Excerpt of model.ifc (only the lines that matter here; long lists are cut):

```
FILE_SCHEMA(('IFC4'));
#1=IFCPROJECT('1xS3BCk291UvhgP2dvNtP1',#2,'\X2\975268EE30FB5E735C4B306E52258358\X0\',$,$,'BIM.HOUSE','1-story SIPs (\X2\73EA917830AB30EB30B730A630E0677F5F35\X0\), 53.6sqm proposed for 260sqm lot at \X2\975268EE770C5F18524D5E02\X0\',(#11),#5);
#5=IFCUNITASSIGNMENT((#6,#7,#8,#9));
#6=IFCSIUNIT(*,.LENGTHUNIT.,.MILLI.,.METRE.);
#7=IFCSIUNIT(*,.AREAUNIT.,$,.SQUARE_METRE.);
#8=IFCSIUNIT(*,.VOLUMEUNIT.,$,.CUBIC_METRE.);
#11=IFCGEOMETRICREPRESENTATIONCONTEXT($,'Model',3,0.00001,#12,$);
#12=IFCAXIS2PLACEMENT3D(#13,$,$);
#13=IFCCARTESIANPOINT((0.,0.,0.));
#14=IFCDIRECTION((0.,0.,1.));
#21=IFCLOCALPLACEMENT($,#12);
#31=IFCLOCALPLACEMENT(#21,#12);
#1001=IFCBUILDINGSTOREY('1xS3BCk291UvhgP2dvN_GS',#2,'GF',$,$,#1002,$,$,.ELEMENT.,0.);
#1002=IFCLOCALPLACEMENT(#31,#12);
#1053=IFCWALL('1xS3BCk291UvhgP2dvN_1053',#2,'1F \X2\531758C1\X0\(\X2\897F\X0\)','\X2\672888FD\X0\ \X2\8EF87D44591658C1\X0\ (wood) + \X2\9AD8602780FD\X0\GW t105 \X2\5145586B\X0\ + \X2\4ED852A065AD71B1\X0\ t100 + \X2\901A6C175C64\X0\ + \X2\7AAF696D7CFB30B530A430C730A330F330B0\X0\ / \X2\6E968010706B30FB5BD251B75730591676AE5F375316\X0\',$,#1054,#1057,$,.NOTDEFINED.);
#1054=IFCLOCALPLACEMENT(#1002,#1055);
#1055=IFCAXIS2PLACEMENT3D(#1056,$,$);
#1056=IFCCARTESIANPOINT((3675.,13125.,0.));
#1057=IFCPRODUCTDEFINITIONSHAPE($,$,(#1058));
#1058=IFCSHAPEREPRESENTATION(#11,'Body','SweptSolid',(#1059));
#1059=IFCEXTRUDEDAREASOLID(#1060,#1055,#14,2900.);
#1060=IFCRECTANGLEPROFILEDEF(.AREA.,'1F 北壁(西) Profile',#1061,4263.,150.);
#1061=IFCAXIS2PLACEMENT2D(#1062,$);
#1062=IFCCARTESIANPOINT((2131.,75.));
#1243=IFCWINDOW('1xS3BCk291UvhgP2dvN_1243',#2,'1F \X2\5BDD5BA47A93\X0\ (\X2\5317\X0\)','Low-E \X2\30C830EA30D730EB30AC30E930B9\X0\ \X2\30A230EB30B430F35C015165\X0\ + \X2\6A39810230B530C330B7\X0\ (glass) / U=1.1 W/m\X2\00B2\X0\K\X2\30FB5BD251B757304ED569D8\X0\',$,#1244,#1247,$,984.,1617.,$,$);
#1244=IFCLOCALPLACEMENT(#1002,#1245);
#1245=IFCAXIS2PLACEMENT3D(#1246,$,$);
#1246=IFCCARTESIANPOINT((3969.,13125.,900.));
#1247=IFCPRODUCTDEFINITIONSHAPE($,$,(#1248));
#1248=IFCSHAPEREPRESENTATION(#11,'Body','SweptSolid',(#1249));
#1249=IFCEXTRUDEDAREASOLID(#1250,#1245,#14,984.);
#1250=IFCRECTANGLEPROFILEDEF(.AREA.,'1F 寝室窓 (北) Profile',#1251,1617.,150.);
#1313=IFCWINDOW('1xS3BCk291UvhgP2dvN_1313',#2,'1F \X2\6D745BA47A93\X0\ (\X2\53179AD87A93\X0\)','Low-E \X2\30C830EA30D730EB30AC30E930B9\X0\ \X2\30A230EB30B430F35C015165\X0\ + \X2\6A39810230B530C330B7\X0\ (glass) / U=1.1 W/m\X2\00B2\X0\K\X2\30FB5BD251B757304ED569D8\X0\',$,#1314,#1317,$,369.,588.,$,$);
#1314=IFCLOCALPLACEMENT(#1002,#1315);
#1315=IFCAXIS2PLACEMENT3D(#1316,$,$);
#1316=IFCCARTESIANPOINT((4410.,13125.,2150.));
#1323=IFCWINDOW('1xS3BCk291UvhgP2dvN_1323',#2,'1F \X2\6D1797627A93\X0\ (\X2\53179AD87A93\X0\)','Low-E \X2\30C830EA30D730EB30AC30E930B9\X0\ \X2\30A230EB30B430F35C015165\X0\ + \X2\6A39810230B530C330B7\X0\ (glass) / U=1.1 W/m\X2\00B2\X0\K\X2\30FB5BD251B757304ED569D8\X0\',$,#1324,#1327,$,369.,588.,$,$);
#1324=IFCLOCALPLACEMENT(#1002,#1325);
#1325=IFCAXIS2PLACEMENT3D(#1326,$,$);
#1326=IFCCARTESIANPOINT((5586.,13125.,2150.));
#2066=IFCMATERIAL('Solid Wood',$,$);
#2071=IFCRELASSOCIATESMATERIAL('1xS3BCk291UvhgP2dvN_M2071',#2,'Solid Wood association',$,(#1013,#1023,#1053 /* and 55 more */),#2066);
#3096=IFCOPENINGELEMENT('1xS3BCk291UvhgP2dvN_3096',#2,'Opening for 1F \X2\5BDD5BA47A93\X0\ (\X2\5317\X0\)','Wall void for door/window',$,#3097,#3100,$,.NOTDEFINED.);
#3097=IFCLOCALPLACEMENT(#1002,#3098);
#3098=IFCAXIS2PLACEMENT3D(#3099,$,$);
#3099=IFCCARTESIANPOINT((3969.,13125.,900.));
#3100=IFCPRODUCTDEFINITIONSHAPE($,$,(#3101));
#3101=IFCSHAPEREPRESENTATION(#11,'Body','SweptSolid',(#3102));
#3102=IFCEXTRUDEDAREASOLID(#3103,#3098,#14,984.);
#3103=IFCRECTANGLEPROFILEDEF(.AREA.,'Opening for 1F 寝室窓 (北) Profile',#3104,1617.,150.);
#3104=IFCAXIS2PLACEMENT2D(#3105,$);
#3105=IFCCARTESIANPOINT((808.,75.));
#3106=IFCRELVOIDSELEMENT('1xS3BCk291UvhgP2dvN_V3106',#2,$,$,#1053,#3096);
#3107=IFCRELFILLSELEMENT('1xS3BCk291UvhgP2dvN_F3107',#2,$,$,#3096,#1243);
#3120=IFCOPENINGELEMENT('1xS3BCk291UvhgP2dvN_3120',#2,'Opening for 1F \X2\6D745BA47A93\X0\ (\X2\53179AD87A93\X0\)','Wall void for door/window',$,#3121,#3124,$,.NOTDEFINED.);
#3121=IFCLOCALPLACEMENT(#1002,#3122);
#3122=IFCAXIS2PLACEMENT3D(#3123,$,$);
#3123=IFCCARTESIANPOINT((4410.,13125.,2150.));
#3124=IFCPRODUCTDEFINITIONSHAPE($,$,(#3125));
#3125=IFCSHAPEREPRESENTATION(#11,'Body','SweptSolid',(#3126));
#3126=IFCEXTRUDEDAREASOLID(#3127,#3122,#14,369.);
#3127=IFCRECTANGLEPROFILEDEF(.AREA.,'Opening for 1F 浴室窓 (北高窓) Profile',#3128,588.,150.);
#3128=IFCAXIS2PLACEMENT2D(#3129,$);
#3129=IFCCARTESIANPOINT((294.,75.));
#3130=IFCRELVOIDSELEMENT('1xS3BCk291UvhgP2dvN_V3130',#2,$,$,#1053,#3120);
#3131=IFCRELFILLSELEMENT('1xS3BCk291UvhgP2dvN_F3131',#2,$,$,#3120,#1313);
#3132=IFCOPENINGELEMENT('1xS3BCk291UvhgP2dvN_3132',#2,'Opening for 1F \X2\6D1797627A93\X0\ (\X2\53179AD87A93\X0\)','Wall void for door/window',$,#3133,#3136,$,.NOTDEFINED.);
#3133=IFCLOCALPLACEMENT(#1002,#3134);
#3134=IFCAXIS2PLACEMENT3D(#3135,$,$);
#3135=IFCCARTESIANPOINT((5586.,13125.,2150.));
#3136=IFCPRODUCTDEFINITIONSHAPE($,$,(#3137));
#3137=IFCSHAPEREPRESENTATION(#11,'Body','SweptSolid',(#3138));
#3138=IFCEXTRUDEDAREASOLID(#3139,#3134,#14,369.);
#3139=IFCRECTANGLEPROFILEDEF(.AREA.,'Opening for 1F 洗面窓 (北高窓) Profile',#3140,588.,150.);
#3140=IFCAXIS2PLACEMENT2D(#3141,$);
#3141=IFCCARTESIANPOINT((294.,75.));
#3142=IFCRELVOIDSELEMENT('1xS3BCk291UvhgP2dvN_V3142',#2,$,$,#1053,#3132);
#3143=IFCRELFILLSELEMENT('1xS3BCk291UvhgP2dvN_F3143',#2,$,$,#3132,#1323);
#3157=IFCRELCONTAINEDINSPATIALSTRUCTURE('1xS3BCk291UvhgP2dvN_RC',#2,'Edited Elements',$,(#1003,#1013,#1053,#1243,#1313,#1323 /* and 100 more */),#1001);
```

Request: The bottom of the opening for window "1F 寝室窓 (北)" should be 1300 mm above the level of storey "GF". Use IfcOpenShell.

```python
import numpy as np
import ifcopenshell
import ifcopenshell.api.geometry
import ifcopenshell.geom
import ifcopenshell.util.element
import ifcopenshell.util.placement
import ifcopenshell.util.shape
import ifcopenshell.util.unit

model = ifcopenshell.open("model.ifc")
unit_scale = ifcopenshell.util.unit.calculate_unit_scale(model)

window = model.by_guid("1xS3BCk291UvhgP2dvN_1243")
opening = window.FillsVoids[0].RelatingOpeningElement
storey = ifcopenshell.util.element.get_container(window, ifc_class="IfcBuildingStorey")
level = ifcopenshell.util.placement.get_local_placement(storey.ObjectPlacement)[2, 3]

# The opening's origin need not be at the sill, so measure its lowest point.
shape = ifcopenshell.geom.create_shape(ifcopenshell.geom.settings(), opening)
bottom = ifcopenshell.util.shape.get_shape_bottom_elevation(shape, shape.geometry) / unit_scale
dz = level + 1300.0 - bottom

shift = np.array([0.0, 0.0, dz])
# The window is not placed relative to its opening, so move both.
for product in (opening, window):
    matrix = ifcopenshell.util.placement.get_local_placement(product.ObjectPlacement)
    matrix[:3, 3] += shift
    ifcopenshell.api.geometry.edit_object_placement(model, product=product, matrix=matrix, is_si=False)

print(f"moved by {dz * unit_scale:+.3f} m")

model.write("model-out.ifc")
```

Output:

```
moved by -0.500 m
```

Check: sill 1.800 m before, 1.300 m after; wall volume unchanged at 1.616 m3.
